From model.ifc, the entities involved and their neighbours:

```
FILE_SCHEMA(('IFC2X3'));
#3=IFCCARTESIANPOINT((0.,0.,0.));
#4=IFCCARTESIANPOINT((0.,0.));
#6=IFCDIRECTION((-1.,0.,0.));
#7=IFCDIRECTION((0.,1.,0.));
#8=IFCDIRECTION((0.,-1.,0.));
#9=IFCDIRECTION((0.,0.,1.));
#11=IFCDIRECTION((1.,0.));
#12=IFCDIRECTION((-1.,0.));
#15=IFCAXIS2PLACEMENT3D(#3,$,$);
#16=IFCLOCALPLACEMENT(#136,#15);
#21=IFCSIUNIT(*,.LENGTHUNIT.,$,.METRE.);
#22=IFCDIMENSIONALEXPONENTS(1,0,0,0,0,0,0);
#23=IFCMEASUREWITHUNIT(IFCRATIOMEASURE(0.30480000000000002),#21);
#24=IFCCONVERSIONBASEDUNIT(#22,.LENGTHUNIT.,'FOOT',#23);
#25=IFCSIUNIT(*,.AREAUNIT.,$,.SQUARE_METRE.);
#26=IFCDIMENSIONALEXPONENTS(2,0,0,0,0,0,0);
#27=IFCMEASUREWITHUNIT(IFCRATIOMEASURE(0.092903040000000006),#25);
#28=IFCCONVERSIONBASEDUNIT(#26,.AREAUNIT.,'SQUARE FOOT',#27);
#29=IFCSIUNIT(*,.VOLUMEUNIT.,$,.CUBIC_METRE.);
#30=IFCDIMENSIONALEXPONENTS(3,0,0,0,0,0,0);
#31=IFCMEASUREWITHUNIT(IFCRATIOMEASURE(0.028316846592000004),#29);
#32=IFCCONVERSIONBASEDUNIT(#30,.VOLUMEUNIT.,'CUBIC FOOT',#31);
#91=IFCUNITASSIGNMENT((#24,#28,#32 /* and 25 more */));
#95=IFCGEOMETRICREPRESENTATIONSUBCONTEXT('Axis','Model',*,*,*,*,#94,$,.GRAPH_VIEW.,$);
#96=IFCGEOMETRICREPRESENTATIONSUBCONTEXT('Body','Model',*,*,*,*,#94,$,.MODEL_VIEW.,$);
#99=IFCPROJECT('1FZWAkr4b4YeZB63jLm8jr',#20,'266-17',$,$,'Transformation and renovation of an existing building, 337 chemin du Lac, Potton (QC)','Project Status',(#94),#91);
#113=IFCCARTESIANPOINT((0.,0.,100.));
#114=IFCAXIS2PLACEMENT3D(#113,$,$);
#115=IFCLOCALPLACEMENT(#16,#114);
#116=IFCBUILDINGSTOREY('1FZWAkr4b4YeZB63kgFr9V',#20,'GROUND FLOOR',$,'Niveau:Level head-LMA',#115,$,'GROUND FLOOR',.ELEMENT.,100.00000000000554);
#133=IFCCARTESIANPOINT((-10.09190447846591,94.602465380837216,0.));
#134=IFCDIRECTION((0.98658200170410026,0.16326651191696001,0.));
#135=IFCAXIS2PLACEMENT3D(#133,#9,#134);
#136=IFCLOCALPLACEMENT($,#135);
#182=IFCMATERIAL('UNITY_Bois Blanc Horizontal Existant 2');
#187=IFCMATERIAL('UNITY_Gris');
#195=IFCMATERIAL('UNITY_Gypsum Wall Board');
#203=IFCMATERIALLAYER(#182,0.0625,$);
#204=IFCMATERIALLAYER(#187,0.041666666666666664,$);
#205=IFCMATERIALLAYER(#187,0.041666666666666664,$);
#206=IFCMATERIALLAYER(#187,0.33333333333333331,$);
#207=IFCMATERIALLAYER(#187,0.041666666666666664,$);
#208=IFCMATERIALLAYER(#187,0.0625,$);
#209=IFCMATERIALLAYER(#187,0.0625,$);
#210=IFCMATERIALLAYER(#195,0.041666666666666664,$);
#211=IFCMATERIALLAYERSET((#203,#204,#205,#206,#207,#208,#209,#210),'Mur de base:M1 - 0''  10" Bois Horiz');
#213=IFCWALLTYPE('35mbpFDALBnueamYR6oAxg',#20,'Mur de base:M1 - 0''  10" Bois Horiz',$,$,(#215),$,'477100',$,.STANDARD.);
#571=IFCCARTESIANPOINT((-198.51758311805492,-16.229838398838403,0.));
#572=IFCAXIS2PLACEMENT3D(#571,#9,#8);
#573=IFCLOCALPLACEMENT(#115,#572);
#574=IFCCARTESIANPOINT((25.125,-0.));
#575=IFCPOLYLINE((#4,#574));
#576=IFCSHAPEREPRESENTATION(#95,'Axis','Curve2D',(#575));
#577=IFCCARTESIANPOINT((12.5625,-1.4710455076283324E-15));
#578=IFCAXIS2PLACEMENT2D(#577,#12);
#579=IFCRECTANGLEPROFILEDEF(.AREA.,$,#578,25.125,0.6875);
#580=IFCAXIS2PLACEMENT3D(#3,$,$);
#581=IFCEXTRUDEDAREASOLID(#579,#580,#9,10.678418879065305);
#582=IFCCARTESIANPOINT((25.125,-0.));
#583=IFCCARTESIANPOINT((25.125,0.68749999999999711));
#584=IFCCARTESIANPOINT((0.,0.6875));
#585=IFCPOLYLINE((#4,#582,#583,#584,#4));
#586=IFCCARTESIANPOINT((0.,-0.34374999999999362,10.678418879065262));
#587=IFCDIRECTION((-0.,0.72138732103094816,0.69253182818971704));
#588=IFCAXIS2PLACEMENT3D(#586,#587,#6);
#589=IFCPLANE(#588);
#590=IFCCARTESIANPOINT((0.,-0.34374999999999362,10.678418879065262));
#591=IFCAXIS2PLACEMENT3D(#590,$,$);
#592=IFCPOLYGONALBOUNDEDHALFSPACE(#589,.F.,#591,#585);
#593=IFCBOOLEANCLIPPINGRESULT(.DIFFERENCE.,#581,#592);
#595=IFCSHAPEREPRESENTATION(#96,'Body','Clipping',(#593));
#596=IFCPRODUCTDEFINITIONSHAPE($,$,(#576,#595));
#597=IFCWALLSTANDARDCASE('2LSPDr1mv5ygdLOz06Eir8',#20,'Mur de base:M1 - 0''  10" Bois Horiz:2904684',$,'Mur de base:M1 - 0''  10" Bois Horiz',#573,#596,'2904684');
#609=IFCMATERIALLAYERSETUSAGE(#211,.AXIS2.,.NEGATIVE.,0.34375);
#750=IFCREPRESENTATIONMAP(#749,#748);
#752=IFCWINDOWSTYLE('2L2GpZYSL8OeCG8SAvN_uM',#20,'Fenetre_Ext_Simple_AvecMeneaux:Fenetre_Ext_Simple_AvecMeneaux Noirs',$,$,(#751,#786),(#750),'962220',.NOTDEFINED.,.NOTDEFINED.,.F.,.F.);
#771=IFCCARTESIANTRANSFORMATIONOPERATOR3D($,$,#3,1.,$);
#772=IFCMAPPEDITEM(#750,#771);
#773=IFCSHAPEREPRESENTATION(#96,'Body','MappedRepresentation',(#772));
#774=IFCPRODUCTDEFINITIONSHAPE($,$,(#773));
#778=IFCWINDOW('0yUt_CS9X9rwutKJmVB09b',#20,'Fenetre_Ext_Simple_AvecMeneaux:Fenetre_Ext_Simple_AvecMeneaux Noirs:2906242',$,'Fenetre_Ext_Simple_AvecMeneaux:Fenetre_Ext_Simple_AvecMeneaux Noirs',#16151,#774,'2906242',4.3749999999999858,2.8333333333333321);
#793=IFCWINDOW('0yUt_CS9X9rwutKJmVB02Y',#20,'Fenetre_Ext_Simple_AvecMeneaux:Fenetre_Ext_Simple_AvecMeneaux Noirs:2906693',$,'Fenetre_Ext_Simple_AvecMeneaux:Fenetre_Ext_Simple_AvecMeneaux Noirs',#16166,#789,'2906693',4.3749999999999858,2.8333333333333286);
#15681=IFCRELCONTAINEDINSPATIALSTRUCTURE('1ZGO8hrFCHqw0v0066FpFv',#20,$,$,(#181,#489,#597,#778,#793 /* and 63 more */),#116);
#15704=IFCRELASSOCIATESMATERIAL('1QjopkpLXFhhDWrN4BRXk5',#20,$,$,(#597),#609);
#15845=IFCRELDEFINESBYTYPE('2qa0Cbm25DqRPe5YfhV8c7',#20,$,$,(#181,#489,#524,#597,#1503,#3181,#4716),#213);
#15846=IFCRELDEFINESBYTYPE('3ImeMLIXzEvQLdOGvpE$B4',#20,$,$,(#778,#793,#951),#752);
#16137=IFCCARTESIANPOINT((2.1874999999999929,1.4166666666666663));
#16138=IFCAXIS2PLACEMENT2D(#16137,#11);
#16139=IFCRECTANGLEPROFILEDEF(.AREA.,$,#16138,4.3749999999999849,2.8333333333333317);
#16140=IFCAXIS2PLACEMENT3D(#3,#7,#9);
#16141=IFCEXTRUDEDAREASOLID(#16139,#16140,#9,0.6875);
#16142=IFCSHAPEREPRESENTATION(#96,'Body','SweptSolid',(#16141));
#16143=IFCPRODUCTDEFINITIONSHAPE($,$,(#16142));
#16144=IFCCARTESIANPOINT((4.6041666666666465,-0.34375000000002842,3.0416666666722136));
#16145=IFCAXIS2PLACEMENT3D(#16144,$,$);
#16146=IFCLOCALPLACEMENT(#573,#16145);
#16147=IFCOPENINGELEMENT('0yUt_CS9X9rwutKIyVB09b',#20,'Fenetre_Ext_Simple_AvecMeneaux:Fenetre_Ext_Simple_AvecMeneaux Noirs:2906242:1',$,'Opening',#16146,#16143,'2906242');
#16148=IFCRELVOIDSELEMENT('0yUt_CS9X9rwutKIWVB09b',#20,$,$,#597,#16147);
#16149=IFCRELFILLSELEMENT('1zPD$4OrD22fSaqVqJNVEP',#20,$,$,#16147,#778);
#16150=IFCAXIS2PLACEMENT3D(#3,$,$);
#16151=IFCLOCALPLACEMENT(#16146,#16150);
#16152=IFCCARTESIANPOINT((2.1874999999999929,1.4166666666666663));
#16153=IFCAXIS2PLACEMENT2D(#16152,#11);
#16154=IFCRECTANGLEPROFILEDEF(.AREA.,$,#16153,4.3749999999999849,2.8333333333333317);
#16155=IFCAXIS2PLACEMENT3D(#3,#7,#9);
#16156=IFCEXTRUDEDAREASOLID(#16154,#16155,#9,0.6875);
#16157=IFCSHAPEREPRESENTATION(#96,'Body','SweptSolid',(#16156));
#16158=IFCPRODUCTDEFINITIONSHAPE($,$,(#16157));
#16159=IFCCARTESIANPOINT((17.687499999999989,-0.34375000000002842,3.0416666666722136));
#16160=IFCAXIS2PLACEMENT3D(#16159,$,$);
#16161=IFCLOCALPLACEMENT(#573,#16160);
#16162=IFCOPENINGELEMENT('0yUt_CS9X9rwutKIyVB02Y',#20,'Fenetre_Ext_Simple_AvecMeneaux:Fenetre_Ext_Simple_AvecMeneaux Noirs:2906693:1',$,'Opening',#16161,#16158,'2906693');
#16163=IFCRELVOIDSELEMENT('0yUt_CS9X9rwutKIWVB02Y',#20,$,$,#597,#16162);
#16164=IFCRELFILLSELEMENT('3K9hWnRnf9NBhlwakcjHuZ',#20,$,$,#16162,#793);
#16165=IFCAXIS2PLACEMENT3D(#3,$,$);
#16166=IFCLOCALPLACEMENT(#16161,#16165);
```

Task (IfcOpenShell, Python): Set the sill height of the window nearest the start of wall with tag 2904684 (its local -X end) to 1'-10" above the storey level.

```python
import numpy as np
import ifcopenshell
import ifcopenshell.api.geometry
import ifcopenshell.geom
import ifcopenshell.util.element
import ifcopenshell.util.placement
import ifcopenshell.util.shape
import ifcopenshell.util.unit

model = ifcopenshell.open("model.ifc")
unit_scale = ifcopenshell.util.unit.calculate_unit_scale(model)

window = model.by_guid("0yUt_CS9X9rwutKJmVB09b")
opening = window.FillsVoids[0].RelatingOpeningElement
storey = ifcopenshell.util.element.get_container(window, ifc_class="IfcBuildingStorey")
level = ifcopenshell.util.placement.get_local_placement(storey.ObjectPlacement)[2, 3]

# The opening's origin need not be at the sill, so measure its lowest point.
shape = ifcopenshell.geom.create_shape(ifcopenshell.geom.settings(), opening)
bottom = ifcopenshell.util.shape.get_shape_bottom_elevation(shape, shape.geometry) / unit_scale
dz = level + 22 * 0.0254 / unit_scale - bottom

shift = np.array([0.0, 0.0, dz])
# The window is placed relative to its opening, so it follows when the opening moves.
matrix = ifcopenshell.util.placement.get_local_placement(opening.ObjectPlacement)
matrix[:3, 3] += shift
ifcopenshell.api.geometry.edit_object_placement(
    model, product=opening, matrix=matrix, is_si=False, should_transform_children=True
)

print(f"moved by {dz * unit_scale:+.3f} m")

model.write("model_rev.ifc")
```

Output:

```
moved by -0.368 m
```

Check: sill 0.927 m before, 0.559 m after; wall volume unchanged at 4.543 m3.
